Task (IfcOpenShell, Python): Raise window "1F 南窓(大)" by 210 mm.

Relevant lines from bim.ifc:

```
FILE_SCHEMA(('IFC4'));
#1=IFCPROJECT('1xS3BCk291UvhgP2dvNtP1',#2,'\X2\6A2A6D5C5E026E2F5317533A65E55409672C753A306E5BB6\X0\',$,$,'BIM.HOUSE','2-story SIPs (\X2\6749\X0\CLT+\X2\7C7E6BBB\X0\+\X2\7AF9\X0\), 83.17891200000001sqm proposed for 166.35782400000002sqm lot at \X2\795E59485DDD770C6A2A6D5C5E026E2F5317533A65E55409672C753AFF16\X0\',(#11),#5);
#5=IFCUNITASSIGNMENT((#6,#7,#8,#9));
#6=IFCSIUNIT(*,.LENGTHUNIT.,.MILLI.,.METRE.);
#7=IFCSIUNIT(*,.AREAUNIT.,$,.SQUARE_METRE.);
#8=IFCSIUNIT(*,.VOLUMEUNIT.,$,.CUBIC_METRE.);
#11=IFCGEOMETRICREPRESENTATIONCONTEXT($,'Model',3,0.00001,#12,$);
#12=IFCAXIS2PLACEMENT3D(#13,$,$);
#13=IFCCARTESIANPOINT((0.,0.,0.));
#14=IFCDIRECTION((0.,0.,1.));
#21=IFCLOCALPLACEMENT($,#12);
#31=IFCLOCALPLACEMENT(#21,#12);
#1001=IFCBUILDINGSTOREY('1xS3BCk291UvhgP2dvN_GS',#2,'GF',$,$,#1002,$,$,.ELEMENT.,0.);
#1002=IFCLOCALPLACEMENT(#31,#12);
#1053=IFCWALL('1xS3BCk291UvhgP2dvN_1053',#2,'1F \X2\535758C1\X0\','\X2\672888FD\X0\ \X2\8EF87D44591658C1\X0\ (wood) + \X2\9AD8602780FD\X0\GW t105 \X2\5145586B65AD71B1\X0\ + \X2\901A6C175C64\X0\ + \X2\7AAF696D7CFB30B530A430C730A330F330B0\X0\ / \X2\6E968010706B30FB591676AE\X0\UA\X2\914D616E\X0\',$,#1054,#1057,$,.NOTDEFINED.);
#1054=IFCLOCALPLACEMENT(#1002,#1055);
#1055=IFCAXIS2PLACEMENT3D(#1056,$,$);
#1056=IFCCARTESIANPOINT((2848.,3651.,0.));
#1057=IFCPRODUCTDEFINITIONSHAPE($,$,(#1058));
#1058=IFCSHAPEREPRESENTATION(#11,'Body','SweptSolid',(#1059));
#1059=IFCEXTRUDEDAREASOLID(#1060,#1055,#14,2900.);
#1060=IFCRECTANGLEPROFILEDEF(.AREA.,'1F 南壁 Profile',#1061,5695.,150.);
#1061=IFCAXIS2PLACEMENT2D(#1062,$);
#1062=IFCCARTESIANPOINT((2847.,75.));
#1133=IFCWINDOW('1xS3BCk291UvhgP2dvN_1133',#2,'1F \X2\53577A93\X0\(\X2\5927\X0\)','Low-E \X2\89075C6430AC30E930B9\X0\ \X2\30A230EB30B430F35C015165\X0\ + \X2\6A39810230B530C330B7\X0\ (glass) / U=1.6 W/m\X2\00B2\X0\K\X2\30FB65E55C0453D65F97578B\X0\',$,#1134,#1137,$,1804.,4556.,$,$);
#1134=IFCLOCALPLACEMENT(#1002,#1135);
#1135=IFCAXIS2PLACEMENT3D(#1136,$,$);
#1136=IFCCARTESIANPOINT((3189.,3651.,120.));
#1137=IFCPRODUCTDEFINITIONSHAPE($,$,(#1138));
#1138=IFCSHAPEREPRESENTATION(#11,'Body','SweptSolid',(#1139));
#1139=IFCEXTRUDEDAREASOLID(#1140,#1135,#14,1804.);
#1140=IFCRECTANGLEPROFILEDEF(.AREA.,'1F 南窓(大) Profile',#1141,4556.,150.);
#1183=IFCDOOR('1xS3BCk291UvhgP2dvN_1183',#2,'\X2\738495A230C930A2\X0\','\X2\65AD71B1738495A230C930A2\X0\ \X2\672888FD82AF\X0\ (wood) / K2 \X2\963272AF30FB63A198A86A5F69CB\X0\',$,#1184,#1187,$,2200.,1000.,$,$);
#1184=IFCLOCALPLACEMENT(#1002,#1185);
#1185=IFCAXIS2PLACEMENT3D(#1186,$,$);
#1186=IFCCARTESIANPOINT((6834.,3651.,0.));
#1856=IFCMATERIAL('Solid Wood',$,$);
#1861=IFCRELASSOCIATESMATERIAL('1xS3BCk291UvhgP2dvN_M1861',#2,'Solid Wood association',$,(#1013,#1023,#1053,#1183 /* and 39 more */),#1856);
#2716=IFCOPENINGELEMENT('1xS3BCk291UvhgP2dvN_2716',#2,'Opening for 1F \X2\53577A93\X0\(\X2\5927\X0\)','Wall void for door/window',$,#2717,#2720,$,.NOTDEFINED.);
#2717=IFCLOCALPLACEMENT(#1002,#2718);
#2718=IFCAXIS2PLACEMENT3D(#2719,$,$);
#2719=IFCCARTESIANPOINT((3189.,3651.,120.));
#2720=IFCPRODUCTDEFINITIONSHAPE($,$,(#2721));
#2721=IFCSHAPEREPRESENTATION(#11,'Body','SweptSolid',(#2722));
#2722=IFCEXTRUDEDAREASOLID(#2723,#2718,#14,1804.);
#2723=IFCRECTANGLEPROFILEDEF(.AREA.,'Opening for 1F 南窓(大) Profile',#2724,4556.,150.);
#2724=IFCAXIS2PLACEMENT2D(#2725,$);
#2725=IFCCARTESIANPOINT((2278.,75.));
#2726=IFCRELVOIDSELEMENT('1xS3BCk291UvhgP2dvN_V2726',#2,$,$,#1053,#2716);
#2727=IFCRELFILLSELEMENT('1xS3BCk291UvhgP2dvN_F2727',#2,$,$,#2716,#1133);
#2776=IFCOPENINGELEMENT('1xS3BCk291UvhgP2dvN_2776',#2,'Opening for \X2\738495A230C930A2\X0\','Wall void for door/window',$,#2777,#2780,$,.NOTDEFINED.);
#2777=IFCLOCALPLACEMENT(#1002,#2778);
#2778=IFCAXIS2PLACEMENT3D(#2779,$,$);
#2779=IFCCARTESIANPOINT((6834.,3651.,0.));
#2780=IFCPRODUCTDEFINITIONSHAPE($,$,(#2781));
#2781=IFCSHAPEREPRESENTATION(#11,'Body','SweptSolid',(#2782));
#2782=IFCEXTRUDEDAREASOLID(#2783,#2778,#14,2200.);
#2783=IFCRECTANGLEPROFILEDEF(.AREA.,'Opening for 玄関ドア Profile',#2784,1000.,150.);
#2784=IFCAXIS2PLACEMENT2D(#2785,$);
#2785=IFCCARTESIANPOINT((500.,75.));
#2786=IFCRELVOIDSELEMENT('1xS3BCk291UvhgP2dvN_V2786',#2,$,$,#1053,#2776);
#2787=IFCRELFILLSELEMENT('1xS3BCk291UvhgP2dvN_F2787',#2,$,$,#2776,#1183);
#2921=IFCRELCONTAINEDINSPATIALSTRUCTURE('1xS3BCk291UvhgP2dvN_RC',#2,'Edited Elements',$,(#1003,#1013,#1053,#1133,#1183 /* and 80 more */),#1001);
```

```python
import numpy as np
import ifcopenshell
import ifcopenshell.api.geometry
import ifcopenshell.util.placement
import ifcopenshell.util.unit

model = ifcopenshell.open("bim.ifc")
unit_scale = ifcopenshell.util.unit.calculate_unit_scale(model)

window = model.by_guid("1xS3BCk291UvhgP2dvN_1133")
opening = window.FillsVoids[0].RelatingOpeningElement
dz = 0.21 / unit_scale

shift = np.array([0.0, 0.0, dz])
# The window is not placed relative to its opening, so move both.
for product in (opening, window):
    matrix = ifcopenshell.util.placement.get_local_placement(product.ObjectPlacement)
    matrix[:3, 3] += shift
    ifcopenshell.api.geometry.edit_object_placement(model, product=product, matrix=matrix, is_si=False)

print(f"moved by {dz * unit_scale:+.3f} m")

model.write("bim_edited.ifc")
```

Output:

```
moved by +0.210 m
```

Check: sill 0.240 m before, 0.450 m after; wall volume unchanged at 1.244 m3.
